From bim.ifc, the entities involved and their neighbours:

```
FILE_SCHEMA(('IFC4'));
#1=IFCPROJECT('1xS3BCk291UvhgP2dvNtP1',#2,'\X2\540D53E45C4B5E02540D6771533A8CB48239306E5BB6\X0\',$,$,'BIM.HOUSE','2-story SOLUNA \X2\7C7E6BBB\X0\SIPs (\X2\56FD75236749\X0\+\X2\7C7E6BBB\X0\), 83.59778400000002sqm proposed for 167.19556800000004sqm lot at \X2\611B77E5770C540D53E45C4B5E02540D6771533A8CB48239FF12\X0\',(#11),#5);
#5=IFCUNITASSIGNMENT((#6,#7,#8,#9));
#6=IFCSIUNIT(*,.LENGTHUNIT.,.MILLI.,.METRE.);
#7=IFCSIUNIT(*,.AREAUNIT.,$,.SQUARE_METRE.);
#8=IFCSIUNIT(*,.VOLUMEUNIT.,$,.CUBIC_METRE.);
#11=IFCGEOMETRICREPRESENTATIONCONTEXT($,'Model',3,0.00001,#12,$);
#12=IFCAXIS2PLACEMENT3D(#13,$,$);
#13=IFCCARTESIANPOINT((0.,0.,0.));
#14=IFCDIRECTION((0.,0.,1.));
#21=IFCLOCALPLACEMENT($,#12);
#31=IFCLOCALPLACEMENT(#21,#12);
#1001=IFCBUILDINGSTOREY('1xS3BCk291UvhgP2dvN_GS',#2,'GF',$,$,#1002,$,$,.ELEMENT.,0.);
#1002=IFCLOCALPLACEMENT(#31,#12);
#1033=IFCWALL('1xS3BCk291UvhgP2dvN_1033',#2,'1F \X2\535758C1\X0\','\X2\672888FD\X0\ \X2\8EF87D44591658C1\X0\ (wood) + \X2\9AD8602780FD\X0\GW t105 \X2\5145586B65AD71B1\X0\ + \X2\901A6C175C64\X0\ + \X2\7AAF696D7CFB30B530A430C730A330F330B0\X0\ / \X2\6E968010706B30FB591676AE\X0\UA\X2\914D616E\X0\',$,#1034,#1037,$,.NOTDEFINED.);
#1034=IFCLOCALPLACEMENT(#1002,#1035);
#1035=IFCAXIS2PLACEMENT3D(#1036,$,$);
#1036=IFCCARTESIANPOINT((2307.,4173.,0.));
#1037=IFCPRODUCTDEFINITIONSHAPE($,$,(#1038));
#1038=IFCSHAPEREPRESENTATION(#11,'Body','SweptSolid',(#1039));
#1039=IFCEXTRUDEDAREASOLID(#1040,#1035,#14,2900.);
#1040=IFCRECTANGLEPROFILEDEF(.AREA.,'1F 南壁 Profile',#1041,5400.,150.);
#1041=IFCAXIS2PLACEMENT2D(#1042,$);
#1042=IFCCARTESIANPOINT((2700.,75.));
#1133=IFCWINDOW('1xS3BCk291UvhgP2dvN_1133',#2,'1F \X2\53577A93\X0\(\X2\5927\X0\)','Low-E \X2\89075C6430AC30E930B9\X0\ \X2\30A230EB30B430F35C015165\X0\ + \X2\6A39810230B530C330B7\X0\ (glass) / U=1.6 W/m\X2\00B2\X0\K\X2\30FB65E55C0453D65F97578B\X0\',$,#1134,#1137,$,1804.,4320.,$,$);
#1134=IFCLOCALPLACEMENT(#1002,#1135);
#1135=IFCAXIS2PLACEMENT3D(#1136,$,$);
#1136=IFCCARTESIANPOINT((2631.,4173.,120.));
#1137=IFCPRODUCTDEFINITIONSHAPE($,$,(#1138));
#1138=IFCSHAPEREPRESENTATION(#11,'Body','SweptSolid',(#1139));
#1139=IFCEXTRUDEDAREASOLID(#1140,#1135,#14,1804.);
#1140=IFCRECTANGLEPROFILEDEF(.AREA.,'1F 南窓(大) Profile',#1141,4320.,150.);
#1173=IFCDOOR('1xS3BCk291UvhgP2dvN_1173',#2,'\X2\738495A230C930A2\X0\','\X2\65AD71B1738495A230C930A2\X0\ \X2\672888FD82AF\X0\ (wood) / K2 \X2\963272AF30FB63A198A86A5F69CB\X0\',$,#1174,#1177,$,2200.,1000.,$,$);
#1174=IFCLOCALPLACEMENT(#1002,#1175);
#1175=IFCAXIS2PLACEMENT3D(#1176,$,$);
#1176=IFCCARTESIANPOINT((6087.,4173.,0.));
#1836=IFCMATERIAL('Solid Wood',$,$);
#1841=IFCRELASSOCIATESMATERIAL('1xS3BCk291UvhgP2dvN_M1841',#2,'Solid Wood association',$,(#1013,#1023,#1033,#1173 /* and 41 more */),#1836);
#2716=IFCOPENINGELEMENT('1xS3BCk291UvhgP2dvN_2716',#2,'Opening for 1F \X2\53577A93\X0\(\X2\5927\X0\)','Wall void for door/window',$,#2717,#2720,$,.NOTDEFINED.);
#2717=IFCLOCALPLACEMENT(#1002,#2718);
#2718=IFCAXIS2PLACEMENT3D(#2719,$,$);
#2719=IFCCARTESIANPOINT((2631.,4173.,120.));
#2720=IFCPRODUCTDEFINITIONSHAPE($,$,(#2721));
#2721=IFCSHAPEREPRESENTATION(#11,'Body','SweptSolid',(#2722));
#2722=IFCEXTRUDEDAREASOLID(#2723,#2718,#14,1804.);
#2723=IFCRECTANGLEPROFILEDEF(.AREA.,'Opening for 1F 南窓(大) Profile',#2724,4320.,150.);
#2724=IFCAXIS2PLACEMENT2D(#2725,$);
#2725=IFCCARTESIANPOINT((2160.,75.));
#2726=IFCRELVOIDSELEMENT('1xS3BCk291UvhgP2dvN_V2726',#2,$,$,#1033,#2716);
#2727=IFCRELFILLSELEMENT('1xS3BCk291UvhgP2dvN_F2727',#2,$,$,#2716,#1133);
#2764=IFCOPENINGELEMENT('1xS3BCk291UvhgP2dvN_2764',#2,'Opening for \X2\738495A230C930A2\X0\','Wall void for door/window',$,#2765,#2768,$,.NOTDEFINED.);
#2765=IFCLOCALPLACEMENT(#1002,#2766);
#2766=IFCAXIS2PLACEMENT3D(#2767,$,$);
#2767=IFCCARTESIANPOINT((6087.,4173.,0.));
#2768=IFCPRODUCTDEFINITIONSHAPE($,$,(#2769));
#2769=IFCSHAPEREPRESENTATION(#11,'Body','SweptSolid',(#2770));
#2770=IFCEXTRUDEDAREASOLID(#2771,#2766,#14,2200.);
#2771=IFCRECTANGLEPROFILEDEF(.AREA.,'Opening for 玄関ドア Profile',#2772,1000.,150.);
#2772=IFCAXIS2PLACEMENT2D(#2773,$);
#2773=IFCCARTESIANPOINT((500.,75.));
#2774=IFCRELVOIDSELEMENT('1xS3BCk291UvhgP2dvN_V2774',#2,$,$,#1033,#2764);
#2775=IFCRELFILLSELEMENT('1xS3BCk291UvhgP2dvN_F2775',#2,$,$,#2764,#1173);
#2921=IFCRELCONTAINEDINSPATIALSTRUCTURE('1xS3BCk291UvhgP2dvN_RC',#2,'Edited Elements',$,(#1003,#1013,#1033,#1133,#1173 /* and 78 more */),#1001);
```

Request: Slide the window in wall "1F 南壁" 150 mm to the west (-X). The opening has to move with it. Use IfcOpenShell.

```python
import ifcopenshell
import ifcopenshell.api.geometry
import ifcopenshell.util.placement
import ifcopenshell.util.unit

model = ifcopenshell.open("bim.ifc")
unit_scale = ifcopenshell.util.unit.calculate_unit_scale(model)

window = model.by_id(1133)
opening = window.FillsVoids[0].RelatingOpeningElement
wall = opening.VoidsElements[0].RelatingBuildingElement

wall_matrix = ifcopenshell.util.placement.get_local_placement(wall.ObjectPlacement)
shift = wall_matrix[:3, 0] * -0.15 / unit_scale
before = ifcopenshell.util.placement.get_local_placement(window.ObjectPlacement)[:3, 3].copy()

# The window is not placed relative to its opening, so move both.
for product in (opening, window):
    matrix = ifcopenshell.util.placement.get_local_placement(product.ObjectPlacement)
    matrix[:3, 3] += shift
    ifcopenshell.api.geometry.edit_object_placement(model, product=product, matrix=matrix, is_si=False)

after = ifcopenshell.util.placement.get_local_placement(window.ObjectPlacement)[:3, 3]
print("window moved by", (after - before).round(3) + 0.0)

model.write("bim_rev.ifc")
```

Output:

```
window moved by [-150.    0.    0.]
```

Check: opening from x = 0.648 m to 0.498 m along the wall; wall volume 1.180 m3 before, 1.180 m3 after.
